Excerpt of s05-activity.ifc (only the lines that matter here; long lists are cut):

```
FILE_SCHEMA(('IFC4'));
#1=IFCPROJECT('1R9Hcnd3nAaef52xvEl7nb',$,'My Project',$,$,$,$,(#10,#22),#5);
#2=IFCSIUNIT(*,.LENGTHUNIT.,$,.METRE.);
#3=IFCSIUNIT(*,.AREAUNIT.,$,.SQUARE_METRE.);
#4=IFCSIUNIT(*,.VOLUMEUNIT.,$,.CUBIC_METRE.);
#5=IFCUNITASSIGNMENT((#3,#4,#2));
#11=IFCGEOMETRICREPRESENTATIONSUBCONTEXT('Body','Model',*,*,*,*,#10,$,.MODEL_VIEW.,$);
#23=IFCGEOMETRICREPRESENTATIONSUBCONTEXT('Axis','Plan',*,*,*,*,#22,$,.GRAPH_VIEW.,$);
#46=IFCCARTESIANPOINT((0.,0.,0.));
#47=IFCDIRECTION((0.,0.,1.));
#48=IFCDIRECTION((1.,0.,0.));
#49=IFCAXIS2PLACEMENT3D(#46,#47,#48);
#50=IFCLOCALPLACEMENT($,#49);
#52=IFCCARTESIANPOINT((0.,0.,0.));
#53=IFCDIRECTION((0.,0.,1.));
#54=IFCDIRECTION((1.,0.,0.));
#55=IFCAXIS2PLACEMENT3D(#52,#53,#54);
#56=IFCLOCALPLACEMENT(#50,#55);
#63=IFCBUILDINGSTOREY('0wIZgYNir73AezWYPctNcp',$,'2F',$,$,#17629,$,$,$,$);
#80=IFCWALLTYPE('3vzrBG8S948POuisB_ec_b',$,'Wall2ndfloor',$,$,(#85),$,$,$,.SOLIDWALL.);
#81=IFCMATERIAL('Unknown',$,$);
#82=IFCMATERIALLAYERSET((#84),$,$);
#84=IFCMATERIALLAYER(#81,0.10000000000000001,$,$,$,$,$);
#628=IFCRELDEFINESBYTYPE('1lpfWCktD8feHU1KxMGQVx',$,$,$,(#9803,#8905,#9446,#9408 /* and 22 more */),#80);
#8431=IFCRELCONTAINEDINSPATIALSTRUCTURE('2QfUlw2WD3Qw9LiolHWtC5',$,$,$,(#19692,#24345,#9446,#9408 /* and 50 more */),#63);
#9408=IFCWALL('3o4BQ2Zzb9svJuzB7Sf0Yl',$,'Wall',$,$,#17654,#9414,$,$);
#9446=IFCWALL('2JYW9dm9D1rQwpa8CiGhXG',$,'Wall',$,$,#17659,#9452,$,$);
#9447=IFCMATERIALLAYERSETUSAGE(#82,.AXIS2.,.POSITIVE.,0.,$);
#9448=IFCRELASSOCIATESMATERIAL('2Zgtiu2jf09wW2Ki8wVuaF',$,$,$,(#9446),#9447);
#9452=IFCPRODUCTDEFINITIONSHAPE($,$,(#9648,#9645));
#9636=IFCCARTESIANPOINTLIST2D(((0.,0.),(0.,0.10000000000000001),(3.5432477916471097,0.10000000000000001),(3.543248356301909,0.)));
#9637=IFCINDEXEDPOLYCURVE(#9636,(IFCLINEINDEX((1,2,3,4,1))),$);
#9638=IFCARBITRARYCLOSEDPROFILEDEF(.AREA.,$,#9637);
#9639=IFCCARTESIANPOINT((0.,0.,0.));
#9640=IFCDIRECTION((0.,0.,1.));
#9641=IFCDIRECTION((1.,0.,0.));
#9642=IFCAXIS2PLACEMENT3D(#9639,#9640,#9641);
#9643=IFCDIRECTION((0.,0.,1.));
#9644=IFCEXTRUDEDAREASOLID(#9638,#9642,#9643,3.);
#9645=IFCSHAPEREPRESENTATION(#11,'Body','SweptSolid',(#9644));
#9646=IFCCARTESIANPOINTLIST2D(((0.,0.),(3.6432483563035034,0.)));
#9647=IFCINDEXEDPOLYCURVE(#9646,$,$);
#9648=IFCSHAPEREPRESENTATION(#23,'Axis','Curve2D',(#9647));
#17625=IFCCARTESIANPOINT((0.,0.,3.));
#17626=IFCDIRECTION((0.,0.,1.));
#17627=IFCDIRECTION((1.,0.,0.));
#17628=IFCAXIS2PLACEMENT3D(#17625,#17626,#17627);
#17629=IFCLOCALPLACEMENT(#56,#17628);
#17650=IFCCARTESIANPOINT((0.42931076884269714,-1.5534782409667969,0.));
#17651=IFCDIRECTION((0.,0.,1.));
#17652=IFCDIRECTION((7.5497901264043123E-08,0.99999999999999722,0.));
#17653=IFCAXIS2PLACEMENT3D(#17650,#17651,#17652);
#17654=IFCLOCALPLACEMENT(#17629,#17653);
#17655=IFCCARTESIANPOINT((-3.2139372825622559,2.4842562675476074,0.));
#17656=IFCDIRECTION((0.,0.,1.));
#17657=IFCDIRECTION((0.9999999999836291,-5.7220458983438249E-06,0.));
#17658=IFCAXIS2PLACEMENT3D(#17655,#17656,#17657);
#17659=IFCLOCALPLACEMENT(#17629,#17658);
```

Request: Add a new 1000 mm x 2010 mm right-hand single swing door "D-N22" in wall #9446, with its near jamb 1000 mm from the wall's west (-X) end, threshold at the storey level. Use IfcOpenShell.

```python
import numpy as np
import ifcopenshell
import ifcopenshell.api.feature
import ifcopenshell.api.geometry
import ifcopenshell.api.root
import ifcopenshell.api.spatial
import ifcopenshell.geom
import ifcopenshell.util.element
import ifcopenshell.util.placement
import ifcopenshell.util.representation
import ifcopenshell.util.shape
import ifcopenshell.util.unit

model = ifcopenshell.open("s05-activity.ifc")
unit_scale = ifcopenshell.util.unit.calculate_unit_scale(model)
settings = ifcopenshell.geom.settings()


def volume(element):
    """Net volume in cubic metres, openings subtracted."""
    shape = ifcopenshell.geom.create_shape(settings, element)
    return ifcopenshell.util.shape.get_volume(shape.geometry)


wall = model.by_guid("2JYW9dm9D1rQwpa8CiGhXG")
storey = ifcopenshell.util.element.get_container(wall, ifc_class="IfcBuildingStorey")
context = ifcopenshell.util.representation.get_context(model, "Model", "Body", "MODEL_VIEW")
before = volume(wall)

width, height, from_end, sill = 1, 2.01, 1, 0.0  # metres

# The wall runs along its own X axis, and the end named is its -X end.
wall_shape = ifcopenshell.geom.create_shape(settings, wall)
x, y, z = ifcopenshell.util.shape.get_vertices(wall_shape.geometry).T
start = x.min() + from_end
face, thickness = float(y.min()), float(y.max() - y.min())
wall_matrix = ifcopenshell.util.placement.get_local_placement(wall.ObjectPlacement)
level = ifcopenshell.util.placement.get_local_placement(storey.ObjectPlacement)[2, 3]


def in_wall(x, y):
    """Placement at x, y metres in the wall's axes, at sill height."""
    matrix = wall_matrix.copy()
    matrix[:, 3] = wall_matrix @ np.array([x / unit_scale, y / unit_scale, 0.0, 1.0])
    matrix[2, 3] = level + sill / unit_scale
    return matrix


# Opening: a box that overshoots both wall faces by 50 mm.
opening = ifcopenshell.api.root.create_entity(model, ifc_class="IfcOpeningElement", predefined_type="OPENING")
box = ifcopenshell.api.geometry.add_wall_representation(
    model, context=context, length=width, height=height, thickness=thickness + 0.1
)
ifcopenshell.api.geometry.assign_representation(model, product=opening, representation=box)
ifcopenshell.api.geometry.edit_object_placement(model, product=opening, matrix=in_wall(start, face - 0.05), is_si=False)
ifcopenshell.api.feature.add_feature(model, feature=opening, element=wall)

door = ifcopenshell.api.root.create_entity(model, ifc_class="IfcDoor", name="D-N22", predefined_type="DOOR")
door.OverallWidth, door.OverallHeight = width / unit_scale, height / unit_scale
door.OperationType = "SINGLE_SWING_RIGHT"
body = ifcopenshell.api.geometry.add_door_representation(
    model,
    context=context,
    overall_width=door.OverallWidth,
    overall_height=door.OverallHeight,
    operation_type="SINGLE_SWING_RIGHT",
    lining_properties={"LiningDepth": thickness / unit_scale, "ThresholdDepth": thickness / unit_scale},
)
ifcopenshell.api.geometry.assign_representation(model, product=door, representation=body)
ifcopenshell.api.spatial.assign_container(model, products=[door], relating_structure=storey)
ifcopenshell.api.feature.add_filling(model, opening=opening, element=door)

# The lining spans the wall, so the door starts at the wall face.
ifcopenshell.api.geometry.edit_object_placement(model, product=door, matrix=in_wall(start, face), is_si=False)

after = volume(wall)

print(f"wall volume {before:.3f} -> {after:.3f} m3")

model.write("s05-activity_rev.ifc")
```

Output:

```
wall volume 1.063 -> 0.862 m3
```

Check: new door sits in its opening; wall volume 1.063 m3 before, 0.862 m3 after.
